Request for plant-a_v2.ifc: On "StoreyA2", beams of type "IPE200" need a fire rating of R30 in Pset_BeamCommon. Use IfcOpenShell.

First a look at what the model holds.

```python
import ifcopenshell
import ifcopenshell.util.element

model = ifcopenshell.open("plant-a_v2.ifc")
print(model.schema)
storey = next(s for s in model.by_type("IfcBuildingStorey") if s.Name == "StoreyA2")
beams = [e for e in ifcopenshell.util.element.get_decomposition(storey) if e.is_a("IfcBeam")]
seen = {}
for e in beams:
    element_type = ifcopenshell.util.element.get_type(e)
    key = (element_type.Name if element_type != e and element_type else None, ifcopenshell.util.element.get_pset(e, "Pset_BeamCommon", "FireRating"))
    seen[key] = seen.get(key, 0) + 1
for (name, value), count in sorted(seen.items(), key=str):
    print(count, "x", name, "|", value)
```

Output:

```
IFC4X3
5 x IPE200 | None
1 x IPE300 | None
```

```python
import ifcopenshell
import ifcopenshell.api.pset
import ifcopenshell.util.element

model = ifcopenshell.open("plant-a_v2.ifc")

storey = next(s for s in model.by_type("IfcBuildingStorey") if s.Name == "StoreyA2")
beams = [e for e in ifcopenshell.util.element.get_decomposition(storey) if e.is_a("IfcBeam")]

count = 0
for e in beams:
    element_type = ifcopenshell.util.element.get_type(e)
    if element_type in (None, e) or element_type.Name != "IPE200":
        continue
    # add_pset returns the element's existing set when there is one.
    pset = ifcopenshell.api.pset.add_pset(model, product=e, name="Pset_BeamCommon")
    ifcopenshell.api.pset.edit_pset(model, pset=pset, properties={"FireRating": "R30"})
    count += 1

print(count, "beams updated")

model.write("plant-a_v2-out.ifc")
```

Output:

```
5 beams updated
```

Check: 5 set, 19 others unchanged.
